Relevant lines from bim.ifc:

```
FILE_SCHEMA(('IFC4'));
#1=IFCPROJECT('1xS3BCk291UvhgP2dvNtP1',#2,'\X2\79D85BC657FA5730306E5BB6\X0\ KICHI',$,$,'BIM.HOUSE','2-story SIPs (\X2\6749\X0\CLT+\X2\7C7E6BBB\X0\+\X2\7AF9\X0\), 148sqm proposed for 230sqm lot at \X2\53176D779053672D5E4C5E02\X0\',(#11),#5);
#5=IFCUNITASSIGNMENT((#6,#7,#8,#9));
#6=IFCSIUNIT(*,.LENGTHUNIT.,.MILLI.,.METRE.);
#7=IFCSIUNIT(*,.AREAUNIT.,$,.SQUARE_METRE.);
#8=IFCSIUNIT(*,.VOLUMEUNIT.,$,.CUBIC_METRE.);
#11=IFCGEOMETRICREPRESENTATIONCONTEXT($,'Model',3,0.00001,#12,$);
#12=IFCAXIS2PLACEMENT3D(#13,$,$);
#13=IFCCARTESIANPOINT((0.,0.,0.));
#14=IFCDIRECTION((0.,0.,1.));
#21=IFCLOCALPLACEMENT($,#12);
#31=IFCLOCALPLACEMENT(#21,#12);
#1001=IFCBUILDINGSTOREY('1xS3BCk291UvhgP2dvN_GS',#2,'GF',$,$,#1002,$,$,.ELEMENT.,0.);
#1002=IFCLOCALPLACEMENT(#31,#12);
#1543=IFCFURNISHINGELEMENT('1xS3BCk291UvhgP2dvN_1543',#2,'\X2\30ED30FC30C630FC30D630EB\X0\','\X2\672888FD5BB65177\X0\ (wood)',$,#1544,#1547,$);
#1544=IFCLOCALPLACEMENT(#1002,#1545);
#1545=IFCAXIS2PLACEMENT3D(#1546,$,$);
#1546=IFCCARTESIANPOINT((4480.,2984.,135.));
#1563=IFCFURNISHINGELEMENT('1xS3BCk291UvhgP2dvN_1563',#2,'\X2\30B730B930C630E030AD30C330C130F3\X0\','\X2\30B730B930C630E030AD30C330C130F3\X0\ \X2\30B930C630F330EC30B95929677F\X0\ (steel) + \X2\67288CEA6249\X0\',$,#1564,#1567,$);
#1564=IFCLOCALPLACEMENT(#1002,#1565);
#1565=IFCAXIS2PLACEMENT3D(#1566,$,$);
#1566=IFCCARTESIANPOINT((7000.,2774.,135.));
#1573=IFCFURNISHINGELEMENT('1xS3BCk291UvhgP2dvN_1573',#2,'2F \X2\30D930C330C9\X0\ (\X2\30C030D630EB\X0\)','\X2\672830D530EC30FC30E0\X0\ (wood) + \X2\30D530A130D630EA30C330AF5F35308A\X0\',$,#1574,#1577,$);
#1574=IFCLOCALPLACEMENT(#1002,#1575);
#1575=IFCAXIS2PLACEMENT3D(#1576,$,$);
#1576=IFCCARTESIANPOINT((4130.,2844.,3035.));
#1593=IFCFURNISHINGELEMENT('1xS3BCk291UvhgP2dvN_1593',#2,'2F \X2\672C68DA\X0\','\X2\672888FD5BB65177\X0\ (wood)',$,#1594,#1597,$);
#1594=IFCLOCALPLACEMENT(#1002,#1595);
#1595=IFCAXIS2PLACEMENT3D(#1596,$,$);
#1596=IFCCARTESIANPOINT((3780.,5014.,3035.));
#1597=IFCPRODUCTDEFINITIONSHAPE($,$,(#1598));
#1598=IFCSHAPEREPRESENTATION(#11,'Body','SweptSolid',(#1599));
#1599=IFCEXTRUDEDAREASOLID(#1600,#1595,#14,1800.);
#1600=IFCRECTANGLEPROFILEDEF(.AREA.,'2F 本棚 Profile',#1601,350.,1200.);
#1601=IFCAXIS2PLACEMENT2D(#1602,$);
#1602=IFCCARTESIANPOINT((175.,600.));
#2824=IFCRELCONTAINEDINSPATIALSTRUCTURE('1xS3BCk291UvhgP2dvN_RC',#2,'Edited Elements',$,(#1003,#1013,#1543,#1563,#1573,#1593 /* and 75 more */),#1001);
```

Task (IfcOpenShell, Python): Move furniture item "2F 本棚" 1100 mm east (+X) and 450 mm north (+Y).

```python
import ifcopenshell
import ifcopenshell.api.geometry
import ifcopenshell.util.placement
import ifcopenshell.util.unit

model = ifcopenshell.open("bim.ifc")
unit_scale = ifcopenshell.util.unit.calculate_unit_scale(model)

item = model.by_guid("1xS3BCk291UvhgP2dvN_1593")
matrix = ifcopenshell.util.placement.get_local_placement(item.ObjectPlacement)
matrix[0, 3] += 1.1 / unit_scale
matrix[1, 3] += 0.45 / unit_scale
ifcopenshell.api.geometry.edit_object_placement(model, product=item, matrix=matrix, is_si=False)

print(ifcopenshell.util.placement.get_local_placement(item.ObjectPlacement).round(3) + 0.0)

model.write("bim_v2.ifc")
```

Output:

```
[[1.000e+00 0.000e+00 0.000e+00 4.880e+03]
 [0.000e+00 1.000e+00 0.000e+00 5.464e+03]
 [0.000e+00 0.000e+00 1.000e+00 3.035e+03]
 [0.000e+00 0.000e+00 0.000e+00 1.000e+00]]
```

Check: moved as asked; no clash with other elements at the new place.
